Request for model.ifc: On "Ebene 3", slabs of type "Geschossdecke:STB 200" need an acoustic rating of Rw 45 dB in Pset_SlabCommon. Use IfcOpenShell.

First a look at what the model holds.

```python
import ifcopenshell
import ifcopenshell.util.element

model = ifcopenshell.open("model.ifc")
print(model.schema)
storey = next(s for s in model.by_type("IfcBuildingStorey") if s.Name == "Ebene 3")
slabs = [e for e in ifcopenshell.util.element.get_decomposition(storey) if e.is_a("IfcSlab")]
seen = {}
for e in slabs:
    element_type = ifcopenshell.util.element.get_type(e)
    key = (element_type.Name if element_type != e and element_type else None, ifcopenshell.util.element.get_pset(e, "Pset_SlabCommon", "AcousticRating"))
    seen[key] = seen.get(key, 0) + 1
for (name, value), count in sorted(seen.items(), key=str):
    print(count, "x", name, "|", value)
```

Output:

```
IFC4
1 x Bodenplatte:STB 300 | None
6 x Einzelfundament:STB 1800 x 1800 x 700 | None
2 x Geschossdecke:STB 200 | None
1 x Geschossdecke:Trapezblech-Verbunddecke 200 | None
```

```python
import ifcopenshell
import ifcopenshell.api.pset
import ifcopenshell.util.element

model = ifcopenshell.open("model.ifc")

storey = next(s for s in model.by_type("IfcBuildingStorey") if s.Name == "Ebene 3")
slabs = [e for e in ifcopenshell.util.element.get_decomposition(storey) if e.is_a("IfcSlab")]

count = 0
for e in slabs:
    element_type = ifcopenshell.util.element.get_type(e)
    if element_type in (None, e) or element_type.Name != "Geschossdecke:STB 200":
        continue
    # add_pset returns the element's existing set when there is one.
    pset = ifcopenshell.api.pset.add_pset(model, product=e, name="Pset_SlabCommon")
    ifcopenshell.api.pset.edit_pset(model, pset=pset, properties={"AcousticRating": "Rw 45 dB"})
    count += 1

print(count, "slabs updated")

model.write("model_v2.ifc")
```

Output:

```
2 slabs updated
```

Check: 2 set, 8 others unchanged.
